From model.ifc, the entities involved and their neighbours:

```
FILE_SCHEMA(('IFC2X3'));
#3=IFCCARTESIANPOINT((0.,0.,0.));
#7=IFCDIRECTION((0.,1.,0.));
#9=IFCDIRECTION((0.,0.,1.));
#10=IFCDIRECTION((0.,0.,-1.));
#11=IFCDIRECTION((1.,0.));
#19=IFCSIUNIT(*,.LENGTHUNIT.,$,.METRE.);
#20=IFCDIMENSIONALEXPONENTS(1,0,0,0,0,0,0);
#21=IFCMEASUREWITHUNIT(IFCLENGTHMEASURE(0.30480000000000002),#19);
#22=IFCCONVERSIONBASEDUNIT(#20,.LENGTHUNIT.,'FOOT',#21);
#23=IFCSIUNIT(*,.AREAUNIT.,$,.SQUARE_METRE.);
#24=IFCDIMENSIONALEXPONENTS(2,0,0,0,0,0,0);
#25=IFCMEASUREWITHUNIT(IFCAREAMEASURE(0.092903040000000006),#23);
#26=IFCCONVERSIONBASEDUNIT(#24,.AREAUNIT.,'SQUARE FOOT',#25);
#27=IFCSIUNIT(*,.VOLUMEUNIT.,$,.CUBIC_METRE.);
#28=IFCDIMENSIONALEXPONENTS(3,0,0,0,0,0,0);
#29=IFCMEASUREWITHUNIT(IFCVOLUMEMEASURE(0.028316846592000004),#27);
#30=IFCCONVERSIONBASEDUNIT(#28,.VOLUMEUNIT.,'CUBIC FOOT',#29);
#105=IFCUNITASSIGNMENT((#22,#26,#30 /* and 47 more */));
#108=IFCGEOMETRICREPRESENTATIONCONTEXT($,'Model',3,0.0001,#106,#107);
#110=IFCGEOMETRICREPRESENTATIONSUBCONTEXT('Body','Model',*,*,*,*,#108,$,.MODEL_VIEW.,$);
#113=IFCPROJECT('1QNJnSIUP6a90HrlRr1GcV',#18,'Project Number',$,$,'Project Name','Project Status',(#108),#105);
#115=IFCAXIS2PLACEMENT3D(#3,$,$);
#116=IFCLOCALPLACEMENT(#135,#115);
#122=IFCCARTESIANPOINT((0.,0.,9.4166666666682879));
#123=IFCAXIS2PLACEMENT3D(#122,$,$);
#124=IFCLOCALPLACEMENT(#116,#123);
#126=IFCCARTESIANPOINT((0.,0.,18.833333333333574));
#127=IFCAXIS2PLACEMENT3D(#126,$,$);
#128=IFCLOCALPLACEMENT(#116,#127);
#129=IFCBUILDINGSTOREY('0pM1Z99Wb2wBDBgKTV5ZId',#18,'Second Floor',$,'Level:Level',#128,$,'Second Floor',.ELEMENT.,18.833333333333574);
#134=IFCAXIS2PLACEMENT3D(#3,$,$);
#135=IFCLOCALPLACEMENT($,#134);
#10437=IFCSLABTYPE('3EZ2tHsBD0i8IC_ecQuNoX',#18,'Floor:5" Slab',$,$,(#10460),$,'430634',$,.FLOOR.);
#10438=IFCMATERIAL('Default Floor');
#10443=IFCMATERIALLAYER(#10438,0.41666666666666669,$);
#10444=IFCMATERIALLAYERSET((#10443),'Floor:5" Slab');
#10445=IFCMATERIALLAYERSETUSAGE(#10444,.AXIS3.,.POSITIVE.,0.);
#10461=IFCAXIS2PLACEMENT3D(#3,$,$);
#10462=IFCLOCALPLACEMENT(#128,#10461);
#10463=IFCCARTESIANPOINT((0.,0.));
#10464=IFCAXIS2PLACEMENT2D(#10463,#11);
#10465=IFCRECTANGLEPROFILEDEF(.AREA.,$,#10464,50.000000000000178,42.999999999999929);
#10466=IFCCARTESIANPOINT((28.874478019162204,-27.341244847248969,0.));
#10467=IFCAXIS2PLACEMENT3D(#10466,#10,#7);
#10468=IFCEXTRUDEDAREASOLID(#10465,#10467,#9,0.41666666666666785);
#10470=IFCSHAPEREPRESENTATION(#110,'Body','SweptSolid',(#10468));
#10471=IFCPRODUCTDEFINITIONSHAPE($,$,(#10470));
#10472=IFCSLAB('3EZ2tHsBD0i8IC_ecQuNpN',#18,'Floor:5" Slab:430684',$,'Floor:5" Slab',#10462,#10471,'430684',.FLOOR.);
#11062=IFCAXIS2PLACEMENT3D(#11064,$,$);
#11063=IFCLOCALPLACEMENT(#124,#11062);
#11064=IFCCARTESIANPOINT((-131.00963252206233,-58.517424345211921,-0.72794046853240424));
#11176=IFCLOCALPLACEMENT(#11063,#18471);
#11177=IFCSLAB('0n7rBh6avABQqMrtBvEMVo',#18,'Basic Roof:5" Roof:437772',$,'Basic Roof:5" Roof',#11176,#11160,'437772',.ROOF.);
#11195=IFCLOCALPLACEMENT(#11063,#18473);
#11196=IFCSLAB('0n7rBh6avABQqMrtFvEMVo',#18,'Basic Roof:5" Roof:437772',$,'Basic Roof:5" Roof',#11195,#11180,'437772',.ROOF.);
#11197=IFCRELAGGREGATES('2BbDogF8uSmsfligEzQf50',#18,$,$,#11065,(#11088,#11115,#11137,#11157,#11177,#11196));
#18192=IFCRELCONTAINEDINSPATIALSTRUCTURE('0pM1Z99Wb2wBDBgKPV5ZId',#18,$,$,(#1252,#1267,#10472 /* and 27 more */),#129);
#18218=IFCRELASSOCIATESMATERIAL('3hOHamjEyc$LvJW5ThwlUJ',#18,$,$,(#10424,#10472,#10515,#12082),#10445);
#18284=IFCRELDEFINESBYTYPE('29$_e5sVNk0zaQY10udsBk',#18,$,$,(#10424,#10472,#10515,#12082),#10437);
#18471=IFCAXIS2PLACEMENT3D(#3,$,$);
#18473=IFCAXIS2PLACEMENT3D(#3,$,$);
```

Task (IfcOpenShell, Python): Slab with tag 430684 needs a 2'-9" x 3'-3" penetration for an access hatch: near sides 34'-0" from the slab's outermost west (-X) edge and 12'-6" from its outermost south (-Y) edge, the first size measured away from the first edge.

```python
import numpy as np
import ifcopenshell
import ifcopenshell.api.feature
import ifcopenshell.api.geometry
import ifcopenshell.api.root
import ifcopenshell.geom
import ifcopenshell.util.placement
import ifcopenshell.util.representation
import ifcopenshell.util.shape
import ifcopenshell.util.unit

model = ifcopenshell.open("model.ifc")
unit_scale = ifcopenshell.util.unit.calculate_unit_scale(model)
settings = ifcopenshell.geom.settings()


def volume(element):
    """Net volume in cubic metres, openings subtracted."""
    shape = ifcopenshell.geom.create_shape(settings, element)
    return ifcopenshell.util.shape.get_volume(shape.geometry)


slab = model.by_id(10472)
before = volume(slab)

# Extent in the slab's own axes, in metres. The edges named are its -X and -Y sides.
slab_shape = ifcopenshell.geom.create_shape(settings, slab)
vertices = ifcopenshell.util.shape.get_vertices(slab_shape.geometry)
x_min, y_min, bottom = vertices.min(axis=0)
top = vertices[:, 2].max()

opening = ifcopenshell.api.root.create_entity(model, ifc_class="IfcOpeningElement", name="Access hatch opening")
context = ifcopenshell.util.representation.get_context(model, "Model", "Body", "MODEL_VIEW")
width, depth = 0.8382, 0.9906
outline = [(0.0, 0.0), (width, 0.0), (width, depth), (0.0, depth), (0.0, 0.0)]
# Overshoot both faces by 50 mm so the cut is clean.
shape = ifcopenshell.api.geometry.add_slab_representation(
    model, context=context, depth=top - bottom + 0.1, polyline=outline
)
ifcopenshell.api.geometry.assign_representation(model, product=opening, representation=shape)

matrix = ifcopenshell.util.placement.get_local_placement(slab.ObjectPlacement)
matrix[:, 3] = matrix @ np.append(np.array([x_min + 10.3632, y_min + 3.81, bottom - 0.05]) / unit_scale, 1.0)
ifcopenshell.api.geometry.edit_object_placement(model, product=opening, matrix=matrix, is_si=False)
ifcopenshell.api.feature.add_feature(model, feature=opening, element=slab)

after = volume(slab)

print(f"slab volume {before:.3f} -> {after:.3f} m3")

model.write("model-out.ifc")
```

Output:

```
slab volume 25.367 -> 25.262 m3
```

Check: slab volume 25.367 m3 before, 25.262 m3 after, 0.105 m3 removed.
